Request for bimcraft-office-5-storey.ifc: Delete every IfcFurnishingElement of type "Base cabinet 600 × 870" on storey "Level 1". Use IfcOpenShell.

First a look at what the model holds.

```python
import ifcopenshell
import ifcopenshell.util.element

model = ifcopenshell.open("bimcraft-office-5-storey.ifc")
print(model.schema)
storey = next(s for s in model.by_type("IfcBuildingStorey") if s.Name == "Level 1")
furniture = [e for e in ifcopenshell.util.element.get_decomposition(storey) if e.is_a("IfcFurnishingElement")]
seen = {}
for e in furniture:
    element_type = ifcopenshell.util.element.get_type(e)
    name = element_type.Name if element_type not in (None, e) else None
    seen[name] = seen.get(name, 0) + 1
for name, count in sorted(seen.items(), key=str):
    print(count, "x", name)
```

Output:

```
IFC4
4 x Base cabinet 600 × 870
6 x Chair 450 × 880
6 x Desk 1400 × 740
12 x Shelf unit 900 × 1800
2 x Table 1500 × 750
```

```python
import ifcopenshell
import ifcopenshell.api.root
import ifcopenshell.util.element

model = ifcopenshell.open("bimcraft-office-5-storey.ifc")

storey = next(s for s in model.by_type("IfcBuildingStorey") if s.Name == "Level 1")
furniture = [e for e in ifcopenshell.util.element.get_decomposition(storey) if e.is_a("IfcFurnishingElement")]
targets = [e for e in furniture if (t := ifcopenshell.util.element.get_type(e)) not in (None, e) and t.Name == "Base cabinet 600 × 870"]

for e in targets:
    ifcopenshell.api.root.remove_product(model, product=e)
print(len(targets), "removed")

model.write("bimcraft-office-5-storey_rev.ifc")
```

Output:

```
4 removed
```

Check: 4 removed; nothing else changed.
